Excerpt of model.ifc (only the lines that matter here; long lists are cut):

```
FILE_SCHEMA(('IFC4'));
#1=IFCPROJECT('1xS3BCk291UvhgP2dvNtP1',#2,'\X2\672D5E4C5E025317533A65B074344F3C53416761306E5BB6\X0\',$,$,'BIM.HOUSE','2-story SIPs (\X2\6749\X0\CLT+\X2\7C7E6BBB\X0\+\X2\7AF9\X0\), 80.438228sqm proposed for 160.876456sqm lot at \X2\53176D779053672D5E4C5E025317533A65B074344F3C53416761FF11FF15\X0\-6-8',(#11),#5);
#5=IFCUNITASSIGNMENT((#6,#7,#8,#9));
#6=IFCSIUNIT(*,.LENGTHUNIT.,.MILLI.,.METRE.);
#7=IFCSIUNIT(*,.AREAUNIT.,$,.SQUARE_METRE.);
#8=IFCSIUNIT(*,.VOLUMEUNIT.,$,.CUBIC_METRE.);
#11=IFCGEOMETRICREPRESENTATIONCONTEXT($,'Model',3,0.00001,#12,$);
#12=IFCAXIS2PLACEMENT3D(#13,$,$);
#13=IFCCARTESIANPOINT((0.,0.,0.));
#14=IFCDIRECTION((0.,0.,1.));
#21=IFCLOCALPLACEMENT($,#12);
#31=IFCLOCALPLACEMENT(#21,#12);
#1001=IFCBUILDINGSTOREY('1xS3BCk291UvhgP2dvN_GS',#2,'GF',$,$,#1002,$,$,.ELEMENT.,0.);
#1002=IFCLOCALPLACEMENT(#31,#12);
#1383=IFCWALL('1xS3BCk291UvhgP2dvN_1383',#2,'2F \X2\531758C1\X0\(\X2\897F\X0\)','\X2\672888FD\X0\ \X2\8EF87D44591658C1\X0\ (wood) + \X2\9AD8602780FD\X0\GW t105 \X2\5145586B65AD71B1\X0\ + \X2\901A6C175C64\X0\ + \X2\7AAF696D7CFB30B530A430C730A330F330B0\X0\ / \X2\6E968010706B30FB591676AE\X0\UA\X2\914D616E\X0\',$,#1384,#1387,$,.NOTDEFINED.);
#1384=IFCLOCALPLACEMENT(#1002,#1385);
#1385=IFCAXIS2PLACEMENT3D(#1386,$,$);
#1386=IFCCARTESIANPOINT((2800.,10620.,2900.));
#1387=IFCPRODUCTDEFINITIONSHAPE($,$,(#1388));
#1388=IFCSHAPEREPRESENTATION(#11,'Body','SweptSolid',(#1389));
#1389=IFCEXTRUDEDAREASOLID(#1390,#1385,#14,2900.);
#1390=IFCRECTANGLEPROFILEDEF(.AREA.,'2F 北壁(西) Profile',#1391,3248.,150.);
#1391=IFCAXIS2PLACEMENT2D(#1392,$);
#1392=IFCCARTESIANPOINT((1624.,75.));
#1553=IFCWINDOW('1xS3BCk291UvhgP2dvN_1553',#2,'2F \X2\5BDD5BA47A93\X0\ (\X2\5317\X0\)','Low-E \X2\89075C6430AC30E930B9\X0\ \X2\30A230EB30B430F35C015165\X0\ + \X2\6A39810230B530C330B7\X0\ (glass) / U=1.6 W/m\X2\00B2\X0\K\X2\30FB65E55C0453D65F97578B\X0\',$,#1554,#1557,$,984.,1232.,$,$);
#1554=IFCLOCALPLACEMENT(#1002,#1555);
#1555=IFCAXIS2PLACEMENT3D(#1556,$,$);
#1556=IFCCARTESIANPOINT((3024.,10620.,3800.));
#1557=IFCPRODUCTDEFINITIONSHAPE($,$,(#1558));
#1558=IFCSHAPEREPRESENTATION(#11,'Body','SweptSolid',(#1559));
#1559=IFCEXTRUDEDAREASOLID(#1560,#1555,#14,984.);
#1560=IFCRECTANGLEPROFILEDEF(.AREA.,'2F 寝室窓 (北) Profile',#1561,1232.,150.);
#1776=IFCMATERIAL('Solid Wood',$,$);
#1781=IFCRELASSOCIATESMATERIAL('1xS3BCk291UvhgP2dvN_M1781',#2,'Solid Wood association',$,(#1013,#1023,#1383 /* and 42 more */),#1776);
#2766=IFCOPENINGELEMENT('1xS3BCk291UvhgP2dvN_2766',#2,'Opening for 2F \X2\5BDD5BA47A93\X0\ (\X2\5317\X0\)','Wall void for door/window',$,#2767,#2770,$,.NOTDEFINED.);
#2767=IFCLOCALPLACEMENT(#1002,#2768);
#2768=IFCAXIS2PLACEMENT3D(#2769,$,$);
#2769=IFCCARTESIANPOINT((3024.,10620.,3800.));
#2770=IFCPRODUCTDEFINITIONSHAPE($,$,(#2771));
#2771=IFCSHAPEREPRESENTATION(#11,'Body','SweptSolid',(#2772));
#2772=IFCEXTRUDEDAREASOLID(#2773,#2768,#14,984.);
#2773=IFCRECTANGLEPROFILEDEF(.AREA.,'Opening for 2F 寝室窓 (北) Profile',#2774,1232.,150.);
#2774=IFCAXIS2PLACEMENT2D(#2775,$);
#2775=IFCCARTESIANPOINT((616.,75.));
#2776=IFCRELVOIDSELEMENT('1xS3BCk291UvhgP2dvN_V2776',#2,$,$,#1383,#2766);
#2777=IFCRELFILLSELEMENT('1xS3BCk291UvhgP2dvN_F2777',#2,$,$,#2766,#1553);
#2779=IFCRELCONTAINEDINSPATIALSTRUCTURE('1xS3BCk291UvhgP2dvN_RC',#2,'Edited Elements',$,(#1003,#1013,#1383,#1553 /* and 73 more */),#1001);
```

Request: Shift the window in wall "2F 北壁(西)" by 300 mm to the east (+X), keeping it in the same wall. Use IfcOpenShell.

```python
import ifcopenshell
import ifcopenshell.api.geometry
import ifcopenshell.util.placement

model = ifcopenshell.open("model.ifc")

window = model.by_guid("1xS3BCk291UvhgP2dvN_1553")
opening = window.FillsVoids[0].RelatingOpeningElement
wall = opening.VoidsElements[0].RelatingBuildingElement

wall_matrix = ifcopenshell.util.placement.get_local_placement(wall.ObjectPlacement)
shift = wall_matrix[:3, 0] * 300.0
before = ifcopenshell.util.placement.get_local_placement(window.ObjectPlacement)[:3, 3].copy()

# The window is not placed relative to its opening, so move both.
for product in (opening, window):
    matrix = ifcopenshell.util.placement.get_local_placement(product.ObjectPlacement)
    matrix[:3, 3] += shift
    ifcopenshell.api.geometry.edit_object_placement(model, product=product, matrix=matrix, is_si=False)

after = ifcopenshell.util.placement.get_local_placement(window.ObjectPlacement)[:3, 3]
print("window moved by", (after - before).round(3) + 0.0)

model.write("model_updated.ifc")
```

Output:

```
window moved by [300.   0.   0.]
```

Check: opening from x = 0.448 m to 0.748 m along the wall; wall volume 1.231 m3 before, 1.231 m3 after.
